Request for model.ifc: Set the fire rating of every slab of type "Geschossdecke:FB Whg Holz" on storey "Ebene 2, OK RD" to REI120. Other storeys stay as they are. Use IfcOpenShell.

First a look at what the model holds.

```python
import ifcopenshell
import ifcopenshell.util.element

model = ifcopenshell.open("model.ifc")
print(model.schema)
storey = next(s for s in model.by_type("IfcBuildingStorey") if s.Name == "Ebene 2, OK RD")
slabs = [e for e in ifcopenshell.util.element.get_decomposition(storey) if e.is_a("IfcSlab")]
seen = {}
for e in slabs:
    element_type = ifcopenshell.util.element.get_type(e)
    key = (element_type.Name if element_type != e and element_type else None, ifcopenshell.util.element.get_pset(e, "Pset_SlabCommon", "FireRating"))
    seen[key] = seen.get(key, 0) + 1
for (name, value), count in sorted(seen.items(), key=str):
    print(count, "x", name, "|", value)
```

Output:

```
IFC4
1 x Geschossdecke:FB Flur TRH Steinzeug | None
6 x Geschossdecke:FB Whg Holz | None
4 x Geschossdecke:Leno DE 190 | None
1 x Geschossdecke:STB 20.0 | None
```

```python
import ifcopenshell
import ifcopenshell.api.pset
import ifcopenshell.util.element

model = ifcopenshell.open("model.ifc")

storey = next(s for s in model.by_type("IfcBuildingStorey") if s.Name == "Ebene 2, OK RD")
slabs = [e for e in ifcopenshell.util.element.get_decomposition(storey) if e.is_a("IfcSlab")]

count = 0
for e in slabs:
    element_type = ifcopenshell.util.element.get_type(e)
    if element_type in (None, e) or element_type.Name != "Geschossdecke:FB Whg Holz":
        continue
    # add_pset returns the element's existing set when there is one.
    pset = ifcopenshell.api.pset.add_pset(model, product=e, name="Pset_SlabCommon")
    ifcopenshell.api.pset.edit_pset(model, pset=pset, properties={"FireRating": "REI120"})
    count += 1

print(count, "slabs updated")

model.write("model_v2.ifc")
```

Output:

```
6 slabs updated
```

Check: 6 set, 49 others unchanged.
